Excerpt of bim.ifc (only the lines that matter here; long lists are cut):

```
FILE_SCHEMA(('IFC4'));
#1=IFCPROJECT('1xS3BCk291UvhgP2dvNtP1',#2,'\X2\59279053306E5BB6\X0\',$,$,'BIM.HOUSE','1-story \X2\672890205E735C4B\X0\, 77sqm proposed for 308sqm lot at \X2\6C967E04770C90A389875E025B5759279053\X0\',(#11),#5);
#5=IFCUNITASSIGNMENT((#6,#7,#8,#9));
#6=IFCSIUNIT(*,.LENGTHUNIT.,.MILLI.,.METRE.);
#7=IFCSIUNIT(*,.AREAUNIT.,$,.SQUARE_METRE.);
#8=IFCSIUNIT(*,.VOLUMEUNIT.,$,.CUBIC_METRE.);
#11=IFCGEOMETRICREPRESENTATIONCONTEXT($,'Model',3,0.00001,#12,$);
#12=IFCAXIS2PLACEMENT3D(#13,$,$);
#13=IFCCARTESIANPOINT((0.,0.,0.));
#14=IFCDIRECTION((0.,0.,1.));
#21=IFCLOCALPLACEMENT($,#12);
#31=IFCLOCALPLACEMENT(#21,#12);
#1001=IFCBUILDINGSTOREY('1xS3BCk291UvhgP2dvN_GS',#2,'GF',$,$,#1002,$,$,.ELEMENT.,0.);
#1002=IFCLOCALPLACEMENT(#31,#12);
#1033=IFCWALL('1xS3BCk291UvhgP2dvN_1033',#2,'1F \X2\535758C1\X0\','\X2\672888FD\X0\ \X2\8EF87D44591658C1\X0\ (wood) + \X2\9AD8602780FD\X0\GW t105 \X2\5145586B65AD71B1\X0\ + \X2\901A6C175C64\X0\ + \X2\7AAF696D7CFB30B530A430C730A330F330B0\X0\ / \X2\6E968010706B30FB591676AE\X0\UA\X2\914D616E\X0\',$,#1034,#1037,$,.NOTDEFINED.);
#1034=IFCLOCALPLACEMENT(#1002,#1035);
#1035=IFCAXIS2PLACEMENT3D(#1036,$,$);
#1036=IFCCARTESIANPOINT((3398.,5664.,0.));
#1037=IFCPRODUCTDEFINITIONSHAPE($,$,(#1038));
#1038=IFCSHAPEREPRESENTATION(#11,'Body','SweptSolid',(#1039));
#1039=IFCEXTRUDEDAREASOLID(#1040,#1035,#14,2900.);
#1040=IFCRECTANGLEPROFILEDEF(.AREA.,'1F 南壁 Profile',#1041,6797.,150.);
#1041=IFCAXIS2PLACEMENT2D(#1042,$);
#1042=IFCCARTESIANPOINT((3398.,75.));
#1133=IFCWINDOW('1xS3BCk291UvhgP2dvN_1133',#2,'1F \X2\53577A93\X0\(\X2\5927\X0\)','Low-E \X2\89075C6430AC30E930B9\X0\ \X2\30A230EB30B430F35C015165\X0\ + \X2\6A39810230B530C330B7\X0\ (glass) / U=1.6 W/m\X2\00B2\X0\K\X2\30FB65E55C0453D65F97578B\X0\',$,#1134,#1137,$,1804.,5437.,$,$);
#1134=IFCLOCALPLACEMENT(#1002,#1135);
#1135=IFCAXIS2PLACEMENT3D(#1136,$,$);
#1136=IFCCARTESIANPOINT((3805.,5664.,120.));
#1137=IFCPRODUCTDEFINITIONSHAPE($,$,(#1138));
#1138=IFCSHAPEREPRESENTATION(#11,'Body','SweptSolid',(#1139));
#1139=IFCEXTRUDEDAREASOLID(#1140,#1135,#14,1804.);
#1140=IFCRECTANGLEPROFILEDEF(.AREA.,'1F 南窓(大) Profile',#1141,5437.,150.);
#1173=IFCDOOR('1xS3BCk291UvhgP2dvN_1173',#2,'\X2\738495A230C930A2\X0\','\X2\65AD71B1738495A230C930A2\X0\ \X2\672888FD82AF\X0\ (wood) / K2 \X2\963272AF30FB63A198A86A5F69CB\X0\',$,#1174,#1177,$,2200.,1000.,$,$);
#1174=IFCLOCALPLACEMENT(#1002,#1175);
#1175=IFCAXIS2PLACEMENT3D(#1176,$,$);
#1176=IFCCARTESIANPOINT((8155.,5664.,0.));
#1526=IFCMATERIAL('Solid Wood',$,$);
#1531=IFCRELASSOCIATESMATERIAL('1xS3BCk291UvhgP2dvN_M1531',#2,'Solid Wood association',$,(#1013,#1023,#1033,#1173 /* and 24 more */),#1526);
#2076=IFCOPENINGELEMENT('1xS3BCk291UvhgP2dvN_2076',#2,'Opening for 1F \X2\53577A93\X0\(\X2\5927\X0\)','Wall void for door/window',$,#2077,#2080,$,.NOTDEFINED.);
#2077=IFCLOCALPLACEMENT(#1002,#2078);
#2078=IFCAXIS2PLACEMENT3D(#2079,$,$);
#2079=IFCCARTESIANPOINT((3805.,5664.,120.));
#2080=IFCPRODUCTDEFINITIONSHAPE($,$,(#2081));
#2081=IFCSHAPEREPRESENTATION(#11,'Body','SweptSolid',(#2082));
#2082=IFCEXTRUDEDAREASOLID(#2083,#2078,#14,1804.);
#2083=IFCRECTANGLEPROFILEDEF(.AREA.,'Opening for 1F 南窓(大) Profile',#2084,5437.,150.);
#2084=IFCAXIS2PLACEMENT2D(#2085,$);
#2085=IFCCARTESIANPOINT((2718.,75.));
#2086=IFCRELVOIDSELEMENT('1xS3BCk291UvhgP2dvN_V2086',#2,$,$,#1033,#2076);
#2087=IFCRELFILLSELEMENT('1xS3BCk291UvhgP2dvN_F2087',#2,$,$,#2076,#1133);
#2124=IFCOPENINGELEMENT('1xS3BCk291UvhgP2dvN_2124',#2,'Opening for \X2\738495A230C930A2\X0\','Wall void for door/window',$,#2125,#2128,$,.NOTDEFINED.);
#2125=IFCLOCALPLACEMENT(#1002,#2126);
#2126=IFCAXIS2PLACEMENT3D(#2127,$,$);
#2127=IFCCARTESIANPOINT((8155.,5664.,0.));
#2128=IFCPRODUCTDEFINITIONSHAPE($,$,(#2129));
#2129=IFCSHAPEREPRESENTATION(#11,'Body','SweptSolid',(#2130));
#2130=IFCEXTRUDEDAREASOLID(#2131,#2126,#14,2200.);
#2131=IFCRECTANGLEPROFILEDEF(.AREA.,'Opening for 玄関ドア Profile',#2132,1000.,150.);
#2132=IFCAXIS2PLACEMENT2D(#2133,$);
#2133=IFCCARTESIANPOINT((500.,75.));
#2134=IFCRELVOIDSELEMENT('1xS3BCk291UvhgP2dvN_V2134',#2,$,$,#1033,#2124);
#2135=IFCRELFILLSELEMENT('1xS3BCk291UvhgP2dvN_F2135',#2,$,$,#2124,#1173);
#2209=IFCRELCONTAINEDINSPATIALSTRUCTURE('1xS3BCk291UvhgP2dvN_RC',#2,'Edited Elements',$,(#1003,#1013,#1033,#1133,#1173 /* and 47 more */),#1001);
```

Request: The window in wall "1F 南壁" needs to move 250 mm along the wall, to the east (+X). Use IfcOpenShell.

```python
import ifcopenshell
import ifcopenshell.api.geometry
import ifcopenshell.util.placement
import ifcopenshell.util.unit

model = ifcopenshell.open("bim.ifc")
unit_scale = ifcopenshell.util.unit.calculate_unit_scale(model)

window = model.by_id(1133)
opening = window.FillsVoids[0].RelatingOpeningElement
wall = opening.VoidsElements[0].RelatingBuildingElement

wall_matrix = ifcopenshell.util.placement.get_local_placement(wall.ObjectPlacement)
shift = wall_matrix[:3, 0] * 0.25 / unit_scale
before = ifcopenshell.util.placement.get_local_placement(window.ObjectPlacement)[:3, 3].copy()

# The window is not placed relative to its opening, so move both.
for product in (opening, window):
    matrix = ifcopenshell.util.placement.get_local_placement(product.ObjectPlacement)
    matrix[:3, 3] += shift
    ifcopenshell.api.geometry.edit_object_placement(model, product=product, matrix=matrix, is_si=False)

after = ifcopenshell.util.placement.get_local_placement(window.ObjectPlacement)[:3, 3]
print("window moved by", (after - before).round(3) + 0.0)

model.write("bim_v2.ifc")
```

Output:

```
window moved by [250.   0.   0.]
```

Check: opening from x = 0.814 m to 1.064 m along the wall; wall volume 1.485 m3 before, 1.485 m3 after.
